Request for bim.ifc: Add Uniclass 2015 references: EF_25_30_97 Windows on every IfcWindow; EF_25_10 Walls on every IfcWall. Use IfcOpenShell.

First a look at what the model holds.

```python
import ifcopenshell

model = ifcopenshell.open("bim.ifc")
print(model.schema)
print("classifications:", [c.Name for c in model.by_type("IfcClassification")])
for ifc_class in ("IfcDoor", "IfcRoof", "IfcStair", "IfcWall", "IfcWindow"):
    print(ifc_class, len(model.by_type(ifc_class)))
```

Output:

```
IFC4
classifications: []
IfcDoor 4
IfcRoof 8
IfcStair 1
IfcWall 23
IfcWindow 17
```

```python
import ifcopenshell
import ifcopenshell.api.classification

model = ifcopenshell.open("bim.ifc")

system = ifcopenshell.api.classification.add_classification(model, classification="Uniclass 2015")

codes = {
    "IfcWindow": ("EF_25_30_97", "Windows"),
    "IfcWall": ("EF_25_10", "Walls"),
}
for ifc_class, (code, name) in codes.items():
    products = model.by_type(ifc_class)
    ifcopenshell.api.classification.add_reference(
        model, products=products, classification=system, identification=code, name=name
    )
    print(code, len(products))

model.write("bim_edited.ifc")
```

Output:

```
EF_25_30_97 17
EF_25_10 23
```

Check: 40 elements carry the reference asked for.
